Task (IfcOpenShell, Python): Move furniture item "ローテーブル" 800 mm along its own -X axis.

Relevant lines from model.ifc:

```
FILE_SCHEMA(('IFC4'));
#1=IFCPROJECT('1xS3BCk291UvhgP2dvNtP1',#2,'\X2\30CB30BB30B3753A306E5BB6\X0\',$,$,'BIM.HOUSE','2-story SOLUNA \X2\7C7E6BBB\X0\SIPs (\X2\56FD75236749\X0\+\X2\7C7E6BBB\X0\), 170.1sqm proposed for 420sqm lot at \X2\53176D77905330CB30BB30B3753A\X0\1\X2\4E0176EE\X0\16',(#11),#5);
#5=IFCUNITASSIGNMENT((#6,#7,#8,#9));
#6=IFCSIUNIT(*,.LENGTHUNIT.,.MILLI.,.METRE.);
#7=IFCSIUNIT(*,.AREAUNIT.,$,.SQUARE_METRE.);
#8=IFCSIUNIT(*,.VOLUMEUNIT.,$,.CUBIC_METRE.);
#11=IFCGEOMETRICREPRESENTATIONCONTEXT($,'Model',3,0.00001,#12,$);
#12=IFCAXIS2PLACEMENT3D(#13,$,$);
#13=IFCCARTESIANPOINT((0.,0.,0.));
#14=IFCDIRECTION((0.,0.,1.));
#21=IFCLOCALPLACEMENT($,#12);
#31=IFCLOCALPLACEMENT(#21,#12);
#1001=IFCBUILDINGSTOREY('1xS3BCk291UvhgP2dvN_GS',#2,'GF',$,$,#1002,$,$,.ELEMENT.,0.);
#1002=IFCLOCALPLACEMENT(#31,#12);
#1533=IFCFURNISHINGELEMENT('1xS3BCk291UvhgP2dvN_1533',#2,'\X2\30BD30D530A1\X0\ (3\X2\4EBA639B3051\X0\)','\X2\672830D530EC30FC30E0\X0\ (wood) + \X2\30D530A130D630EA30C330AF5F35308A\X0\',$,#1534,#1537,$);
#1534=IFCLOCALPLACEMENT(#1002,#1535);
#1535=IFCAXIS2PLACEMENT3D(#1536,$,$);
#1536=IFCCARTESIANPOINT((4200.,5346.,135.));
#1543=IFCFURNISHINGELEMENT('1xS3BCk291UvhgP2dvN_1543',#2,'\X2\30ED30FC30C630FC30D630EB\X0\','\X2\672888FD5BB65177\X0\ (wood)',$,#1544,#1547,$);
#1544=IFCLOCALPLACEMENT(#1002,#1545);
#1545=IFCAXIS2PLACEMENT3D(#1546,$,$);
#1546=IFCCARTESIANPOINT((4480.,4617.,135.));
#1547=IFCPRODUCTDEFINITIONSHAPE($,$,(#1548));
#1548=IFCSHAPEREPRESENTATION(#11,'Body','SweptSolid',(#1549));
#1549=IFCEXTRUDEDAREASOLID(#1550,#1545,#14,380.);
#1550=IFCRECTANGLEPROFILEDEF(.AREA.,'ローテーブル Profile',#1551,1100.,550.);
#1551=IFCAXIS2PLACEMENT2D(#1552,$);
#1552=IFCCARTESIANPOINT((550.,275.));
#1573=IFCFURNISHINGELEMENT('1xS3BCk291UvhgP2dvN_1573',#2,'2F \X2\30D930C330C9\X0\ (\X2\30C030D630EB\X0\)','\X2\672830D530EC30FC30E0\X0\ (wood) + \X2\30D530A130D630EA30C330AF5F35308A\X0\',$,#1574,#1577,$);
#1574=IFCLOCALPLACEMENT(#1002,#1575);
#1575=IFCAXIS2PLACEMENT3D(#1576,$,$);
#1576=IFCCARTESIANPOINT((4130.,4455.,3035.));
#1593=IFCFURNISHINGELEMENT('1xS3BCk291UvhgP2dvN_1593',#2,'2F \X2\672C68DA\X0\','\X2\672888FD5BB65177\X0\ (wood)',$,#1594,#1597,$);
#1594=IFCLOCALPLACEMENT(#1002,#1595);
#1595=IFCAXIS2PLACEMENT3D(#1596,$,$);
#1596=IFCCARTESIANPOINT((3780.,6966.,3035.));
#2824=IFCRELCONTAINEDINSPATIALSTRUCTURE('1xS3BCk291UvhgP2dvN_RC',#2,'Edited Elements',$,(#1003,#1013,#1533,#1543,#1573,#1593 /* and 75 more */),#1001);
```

```python
import ifcopenshell
import ifcopenshell.api.geometry
import ifcopenshell.util.placement
import ifcopenshell.util.unit

model = ifcopenshell.open("model.ifc")
unit_scale = ifcopenshell.util.unit.calculate_unit_scale(model)

item = model.by_guid("1xS3BCk291UvhgP2dvN_1543")
matrix = ifcopenshell.util.placement.get_local_placement(item.ObjectPlacement)
matrix[:3, 3] -= matrix[:3, 0] * 0.8 / unit_scale
ifcopenshell.api.geometry.edit_object_placement(model, product=item, matrix=matrix, is_si=False)

print(ifcopenshell.util.placement.get_local_placement(item.ObjectPlacement).round(3) + 0.0)

model.write("model_edited.ifc")
```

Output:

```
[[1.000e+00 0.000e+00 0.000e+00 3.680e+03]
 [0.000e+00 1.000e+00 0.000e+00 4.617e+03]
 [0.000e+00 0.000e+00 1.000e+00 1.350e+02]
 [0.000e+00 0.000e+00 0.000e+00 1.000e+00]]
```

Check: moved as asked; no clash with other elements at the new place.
